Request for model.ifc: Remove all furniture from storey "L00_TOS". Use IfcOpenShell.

First a look at what the model holds.

```python
import ifcopenshell
import ifcopenshell.util.element

model = ifcopenshell.open("model.ifc")
print(model.schema)
storey = next(s for s in model.by_type("IfcBuildingStorey") if s.Name == "L00_TOS")
furniture = [e for e in ifcopenshell.util.element.get_decomposition(storey) if e.is_a("IfcFurnishingElement")]
seen = {}
for e in furniture:
    element_type = ifcopenshell.util.element.get_type(e)
    name = element_type.Name if element_type not in (None, e) else None
    seen[name] = seen.get(name, 0) + 1
for name, count in sorted(seen.items(), key=str):
    print(count, "x", name)
```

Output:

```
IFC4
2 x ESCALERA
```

```python
import ifcopenshell
import ifcopenshell.api.root
import ifcopenshell.util.element

model = ifcopenshell.open("model.ifc")

storey = next(s for s in model.by_type("IfcBuildingStorey") if s.Name == "L00_TOS")
furniture = [e for e in ifcopenshell.util.element.get_decomposition(storey) if e.is_a("IfcFurnishingElement")]

for e in furniture:
    ifcopenshell.api.root.remove_product(model, product=e)
print(len(furniture), "removed")

model.write("model_v2.ifc")
```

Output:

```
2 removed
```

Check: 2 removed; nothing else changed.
